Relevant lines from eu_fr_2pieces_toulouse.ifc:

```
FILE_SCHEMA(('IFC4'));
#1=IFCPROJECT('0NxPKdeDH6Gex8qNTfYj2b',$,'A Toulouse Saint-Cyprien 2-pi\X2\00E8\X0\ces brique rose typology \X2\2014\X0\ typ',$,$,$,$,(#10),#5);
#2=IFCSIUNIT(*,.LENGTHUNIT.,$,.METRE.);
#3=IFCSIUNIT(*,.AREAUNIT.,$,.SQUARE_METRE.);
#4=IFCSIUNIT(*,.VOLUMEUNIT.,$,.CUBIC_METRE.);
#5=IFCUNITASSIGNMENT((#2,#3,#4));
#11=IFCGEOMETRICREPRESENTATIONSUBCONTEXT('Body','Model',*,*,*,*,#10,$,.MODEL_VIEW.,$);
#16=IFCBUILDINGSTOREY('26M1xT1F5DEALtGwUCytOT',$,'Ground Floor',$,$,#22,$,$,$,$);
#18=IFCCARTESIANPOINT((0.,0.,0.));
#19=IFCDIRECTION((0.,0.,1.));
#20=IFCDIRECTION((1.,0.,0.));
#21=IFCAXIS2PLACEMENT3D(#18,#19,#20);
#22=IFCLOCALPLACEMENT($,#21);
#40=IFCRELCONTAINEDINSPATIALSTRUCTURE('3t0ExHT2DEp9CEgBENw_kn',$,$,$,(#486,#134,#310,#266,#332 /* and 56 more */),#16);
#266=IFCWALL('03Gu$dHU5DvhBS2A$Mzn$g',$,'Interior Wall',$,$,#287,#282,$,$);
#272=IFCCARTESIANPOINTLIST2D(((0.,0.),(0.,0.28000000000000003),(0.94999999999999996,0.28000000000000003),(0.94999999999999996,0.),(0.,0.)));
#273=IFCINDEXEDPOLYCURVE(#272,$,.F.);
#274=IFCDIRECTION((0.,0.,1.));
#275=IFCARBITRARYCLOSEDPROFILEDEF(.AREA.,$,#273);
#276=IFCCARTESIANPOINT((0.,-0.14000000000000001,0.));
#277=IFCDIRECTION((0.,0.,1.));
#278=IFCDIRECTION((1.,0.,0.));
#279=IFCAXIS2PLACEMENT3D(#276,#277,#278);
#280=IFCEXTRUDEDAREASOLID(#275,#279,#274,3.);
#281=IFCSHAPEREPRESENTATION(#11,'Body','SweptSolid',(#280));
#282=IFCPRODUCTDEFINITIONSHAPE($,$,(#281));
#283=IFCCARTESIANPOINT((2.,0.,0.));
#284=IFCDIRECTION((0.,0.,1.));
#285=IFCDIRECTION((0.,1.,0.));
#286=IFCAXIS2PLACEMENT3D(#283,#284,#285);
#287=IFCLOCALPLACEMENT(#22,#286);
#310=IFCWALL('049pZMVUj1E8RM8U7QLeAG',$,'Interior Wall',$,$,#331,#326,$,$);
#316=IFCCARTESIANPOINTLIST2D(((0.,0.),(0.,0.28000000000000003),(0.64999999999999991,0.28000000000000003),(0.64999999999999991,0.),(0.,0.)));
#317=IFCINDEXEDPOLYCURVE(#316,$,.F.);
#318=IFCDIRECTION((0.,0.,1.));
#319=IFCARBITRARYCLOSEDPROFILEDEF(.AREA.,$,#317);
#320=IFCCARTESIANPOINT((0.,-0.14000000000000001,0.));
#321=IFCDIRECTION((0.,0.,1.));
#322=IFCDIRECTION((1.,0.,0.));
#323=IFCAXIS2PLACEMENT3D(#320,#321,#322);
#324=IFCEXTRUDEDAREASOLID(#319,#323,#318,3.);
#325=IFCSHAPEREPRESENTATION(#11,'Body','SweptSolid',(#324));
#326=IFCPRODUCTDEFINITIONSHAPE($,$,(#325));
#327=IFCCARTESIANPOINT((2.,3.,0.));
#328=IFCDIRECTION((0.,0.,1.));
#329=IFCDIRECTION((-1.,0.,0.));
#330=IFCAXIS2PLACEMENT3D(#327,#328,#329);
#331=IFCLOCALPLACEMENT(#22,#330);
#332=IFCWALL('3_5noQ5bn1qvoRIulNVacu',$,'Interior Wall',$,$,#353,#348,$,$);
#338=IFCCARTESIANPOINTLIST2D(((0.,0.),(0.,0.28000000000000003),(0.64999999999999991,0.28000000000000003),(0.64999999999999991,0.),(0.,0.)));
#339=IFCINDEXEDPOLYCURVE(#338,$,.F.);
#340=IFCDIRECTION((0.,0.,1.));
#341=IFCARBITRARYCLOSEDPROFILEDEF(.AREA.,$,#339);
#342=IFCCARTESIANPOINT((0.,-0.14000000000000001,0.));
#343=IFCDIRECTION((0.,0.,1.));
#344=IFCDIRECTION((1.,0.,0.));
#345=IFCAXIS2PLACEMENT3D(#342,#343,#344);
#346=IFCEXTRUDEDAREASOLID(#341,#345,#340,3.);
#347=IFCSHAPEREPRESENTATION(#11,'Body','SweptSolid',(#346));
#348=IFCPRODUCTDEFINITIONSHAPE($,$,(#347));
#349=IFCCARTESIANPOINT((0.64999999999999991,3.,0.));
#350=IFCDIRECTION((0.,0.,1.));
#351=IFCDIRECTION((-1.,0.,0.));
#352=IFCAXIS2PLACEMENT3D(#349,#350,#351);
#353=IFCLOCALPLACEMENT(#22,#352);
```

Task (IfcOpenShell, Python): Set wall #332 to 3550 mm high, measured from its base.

```python
import ifcopenshell
import ifcopenshell.geom
import ifcopenshell.util.representation
import ifcopenshell.util.shape
import ifcopenshell.util.unit

model = ifcopenshell.open("eu_fr_2pieces_toulouse.ifc")
unit_scale = ifcopenshell.util.unit.calculate_unit_scale(model)
settings = ifcopenshell.geom.settings()


def volume(element):
    """Net volume in cubic metres, openings subtracted."""
    shape = ifcopenshell.geom.create_shape(settings, element)
    return ifcopenshell.util.shape.get_volume(shape.geometry)


wall = model.by_guid("3_5noQ5bn1qvoRIulNVacu")
before = volume(wall)

body = ifcopenshell.util.representation.get_representation(wall, "Model", "Body")
solid = body.Items[0]
old_height = solid.Depth
solid.Depth = 3.55 / unit_scale
after = volume(wall)

print(f"height {old_height:g} -> {solid.Depth:g}, volume {before:.3f} -> {after:.3f} m3")

model.write("eu_fr_2pieces_toulouse_edited.ifc")
```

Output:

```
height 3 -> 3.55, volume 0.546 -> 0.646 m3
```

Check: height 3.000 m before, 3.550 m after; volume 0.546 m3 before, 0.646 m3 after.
